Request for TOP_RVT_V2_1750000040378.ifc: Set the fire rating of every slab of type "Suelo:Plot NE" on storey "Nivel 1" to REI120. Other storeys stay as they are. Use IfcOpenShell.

First a look at what the model holds.

```python
import ifcopenshell
import ifcopenshell.util.element

model = ifcopenshell.open("TOP_RVT_V2_1750000040378.ifc")
print(model.schema)
storey = next(s for s in model.by_type("IfcBuildingStorey") if s.Name == "Nivel 1")
slabs = [e for e in ifcopenshell.util.element.get_decomposition(storey) if e.is_a("IfcSlab")]
seen = {}
for e in slabs:
    element_type = ifcopenshell.util.element.get_type(e)
    key = (element_type.Name if element_type != e and element_type else None, ifcopenshell.util.element.get_pset(e, "Pset_SlabCommon", "FireRating"))
    seen[key] = seen.get(key, 0) + 1
for (name, value), count in sorted(seen.items(), key=str):
    print(count, "x", name, "|", value)
```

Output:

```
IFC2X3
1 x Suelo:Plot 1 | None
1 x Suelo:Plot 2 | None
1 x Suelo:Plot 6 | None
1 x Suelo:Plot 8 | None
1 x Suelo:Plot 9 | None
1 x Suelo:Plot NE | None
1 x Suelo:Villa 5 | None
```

```python
import ifcopenshell
import ifcopenshell.api.pset
import ifcopenshell.util.element

model = ifcopenshell.open("TOP_RVT_V2_1750000040378.ifc")

storey = next(s for s in model.by_type("IfcBuildingStorey") if s.Name == "Nivel 1")
slabs = [e for e in ifcopenshell.util.element.get_decomposition(storey) if e.is_a("IfcSlab")]

count = 0
for e in slabs:
    element_type = ifcopenshell.util.element.get_type(e)
    if element_type in (None, e) or element_type.Name != "Suelo:Plot NE":
        continue
    # add_pset returns the element's existing set when there is one.
    pset = ifcopenshell.api.pset.add_pset(model, product=e, name="Pset_SlabCommon")
    ifcopenshell.api.pset.edit_pset(model, pset=pset, properties={"FireRating": "REI120"})
    count += 1

print(count, "slabs updated")

model.write("TOP_RVT_V2_1750000040378_v2.ifc")
```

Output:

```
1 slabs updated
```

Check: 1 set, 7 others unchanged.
